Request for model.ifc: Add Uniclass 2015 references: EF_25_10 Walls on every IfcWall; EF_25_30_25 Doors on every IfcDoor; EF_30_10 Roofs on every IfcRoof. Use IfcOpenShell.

First a look at what the model holds.

```python
import ifcopenshell

model = ifcopenshell.open("model.ifc")
print(model.schema)
print("classifications:", [c.Name for c in model.by_type("IfcClassification")])
for ifc_class in ("IfcDoor", "IfcRoof", "IfcStair", "IfcWall", "IfcWindow"):
    print(ifc_class, len(model.by_type(ifc_class)))
```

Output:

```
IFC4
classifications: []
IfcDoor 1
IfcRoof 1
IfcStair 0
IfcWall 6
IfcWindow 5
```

```python
import ifcopenshell
import ifcopenshell.api.classification

model = ifcopenshell.open("model.ifc")

system = ifcopenshell.api.classification.add_classification(model, classification="Uniclass 2015")

codes = {
    "IfcWall": ("EF_25_10", "Walls"),
    "IfcDoor": ("EF_25_30_25", "Doors"),
    "IfcRoof": ("EF_30_10", "Roofs"),
}
for ifc_class, (code, name) in codes.items():
    products = model.by_type(ifc_class)
    ifcopenshell.api.classification.add_reference(
        model, products=products, classification=system, identification=code, name=name
    )
    print(code, len(products))

model.write("model_rev.ifc")
```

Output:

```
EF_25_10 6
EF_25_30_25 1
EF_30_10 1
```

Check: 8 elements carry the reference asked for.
